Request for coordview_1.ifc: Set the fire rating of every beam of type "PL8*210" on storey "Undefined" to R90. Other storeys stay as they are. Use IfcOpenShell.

First a look at what the model holds.

```python
import ifcopenshell
import ifcopenshell.util.element

model = ifcopenshell.open("coordview_1.ifc")
print(model.schema)
storey = next(s for s in model.by_type("IfcBuildingStorey") if s.Name == "Undefined")
beams = [e for e in ifcopenshell.util.element.get_decomposition(storey) if e.is_a("IfcBeam")]
seen = {}
for e in beams:
    element_type = ifcopenshell.util.element.get_type(e)
    key = (element_type.Name if element_type != e and element_type else None, ifcopenshell.util.element.get_pset(e, "Pset_BeamCommon", "FireRating"))
    seen[key] = seen.get(key, 0) + 1
for (name, value), count in sorted(seen.items(), key=str):
    print(count, "x", name, "|", value)
```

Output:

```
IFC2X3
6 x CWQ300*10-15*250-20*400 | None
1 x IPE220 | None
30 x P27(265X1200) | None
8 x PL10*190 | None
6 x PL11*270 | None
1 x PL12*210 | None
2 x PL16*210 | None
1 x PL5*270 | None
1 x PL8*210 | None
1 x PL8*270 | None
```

```python
import ifcopenshell
import ifcopenshell.api.pset
import ifcopenshell.util.element

model = ifcopenshell.open("coordview_1.ifc")

storey = next(s for s in model.by_type("IfcBuildingStorey") if s.Name == "Undefined")
beams = [e for e in ifcopenshell.util.element.get_decomposition(storey) if e.is_a("IfcBeam")]

count = 0
for e in beams:
    element_type = ifcopenshell.util.element.get_type(e)
    if element_type in (None, e) or element_type.Name != "PL8*210":
        continue
    found = ifcopenshell.util.element.get_pset(e, "Pset_BeamCommon", should_inherit=False)
    if found:
        pset = model.by_id(found["id"])
        if len(ifcopenshell.util.element.get_elements_by_pset(pset)) > 1:
            pset = ifcopenshell.api.pset.unshare_pset(model, products=[e], pset=pset)[0]
    else:
        pset = ifcopenshell.api.pset.add_pset(model, product=e, name="Pset_BeamCommon")
    ifcopenshell.api.pset.edit_pset(model, pset=pset, properties={"FireRating": "R90"})
    count += 1

print(count, "beams updated")

model.write("coordview_1-out.ifc")
```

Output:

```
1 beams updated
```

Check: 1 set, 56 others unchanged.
